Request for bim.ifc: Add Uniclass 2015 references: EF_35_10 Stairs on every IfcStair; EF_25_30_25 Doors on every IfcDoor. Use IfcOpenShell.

First a look at what the model holds.

```python
import ifcopenshell

model = ifcopenshell.open("bim.ifc")
print(model.schema)
print("classifications:", [c.Name for c in model.by_type("IfcClassification")])
for ifc_class in ("IfcDoor", "IfcRoof", "IfcStair", "IfcWall", "IfcWindow"):
    print(ifc_class, len(model.by_type(ifc_class)))
```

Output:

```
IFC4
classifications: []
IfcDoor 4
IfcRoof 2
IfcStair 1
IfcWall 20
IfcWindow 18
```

```python
import ifcopenshell
import ifcopenshell.api.classification

model = ifcopenshell.open("bim.ifc")

system = ifcopenshell.api.classification.add_classification(model, classification="Uniclass 2015")

codes = {
    "IfcStair": ("EF_35_10", "Stairs"),
    "IfcDoor": ("EF_25_30_25", "Doors"),
}
for ifc_class, (code, name) in codes.items():
    products = model.by_type(ifc_class)
    ifcopenshell.api.classification.add_reference(
        model, products=products, classification=system, identification=code, name=name
    )
    print(code, len(products))

model.write("bim-out.ifc")
```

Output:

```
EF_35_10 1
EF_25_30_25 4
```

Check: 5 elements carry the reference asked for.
